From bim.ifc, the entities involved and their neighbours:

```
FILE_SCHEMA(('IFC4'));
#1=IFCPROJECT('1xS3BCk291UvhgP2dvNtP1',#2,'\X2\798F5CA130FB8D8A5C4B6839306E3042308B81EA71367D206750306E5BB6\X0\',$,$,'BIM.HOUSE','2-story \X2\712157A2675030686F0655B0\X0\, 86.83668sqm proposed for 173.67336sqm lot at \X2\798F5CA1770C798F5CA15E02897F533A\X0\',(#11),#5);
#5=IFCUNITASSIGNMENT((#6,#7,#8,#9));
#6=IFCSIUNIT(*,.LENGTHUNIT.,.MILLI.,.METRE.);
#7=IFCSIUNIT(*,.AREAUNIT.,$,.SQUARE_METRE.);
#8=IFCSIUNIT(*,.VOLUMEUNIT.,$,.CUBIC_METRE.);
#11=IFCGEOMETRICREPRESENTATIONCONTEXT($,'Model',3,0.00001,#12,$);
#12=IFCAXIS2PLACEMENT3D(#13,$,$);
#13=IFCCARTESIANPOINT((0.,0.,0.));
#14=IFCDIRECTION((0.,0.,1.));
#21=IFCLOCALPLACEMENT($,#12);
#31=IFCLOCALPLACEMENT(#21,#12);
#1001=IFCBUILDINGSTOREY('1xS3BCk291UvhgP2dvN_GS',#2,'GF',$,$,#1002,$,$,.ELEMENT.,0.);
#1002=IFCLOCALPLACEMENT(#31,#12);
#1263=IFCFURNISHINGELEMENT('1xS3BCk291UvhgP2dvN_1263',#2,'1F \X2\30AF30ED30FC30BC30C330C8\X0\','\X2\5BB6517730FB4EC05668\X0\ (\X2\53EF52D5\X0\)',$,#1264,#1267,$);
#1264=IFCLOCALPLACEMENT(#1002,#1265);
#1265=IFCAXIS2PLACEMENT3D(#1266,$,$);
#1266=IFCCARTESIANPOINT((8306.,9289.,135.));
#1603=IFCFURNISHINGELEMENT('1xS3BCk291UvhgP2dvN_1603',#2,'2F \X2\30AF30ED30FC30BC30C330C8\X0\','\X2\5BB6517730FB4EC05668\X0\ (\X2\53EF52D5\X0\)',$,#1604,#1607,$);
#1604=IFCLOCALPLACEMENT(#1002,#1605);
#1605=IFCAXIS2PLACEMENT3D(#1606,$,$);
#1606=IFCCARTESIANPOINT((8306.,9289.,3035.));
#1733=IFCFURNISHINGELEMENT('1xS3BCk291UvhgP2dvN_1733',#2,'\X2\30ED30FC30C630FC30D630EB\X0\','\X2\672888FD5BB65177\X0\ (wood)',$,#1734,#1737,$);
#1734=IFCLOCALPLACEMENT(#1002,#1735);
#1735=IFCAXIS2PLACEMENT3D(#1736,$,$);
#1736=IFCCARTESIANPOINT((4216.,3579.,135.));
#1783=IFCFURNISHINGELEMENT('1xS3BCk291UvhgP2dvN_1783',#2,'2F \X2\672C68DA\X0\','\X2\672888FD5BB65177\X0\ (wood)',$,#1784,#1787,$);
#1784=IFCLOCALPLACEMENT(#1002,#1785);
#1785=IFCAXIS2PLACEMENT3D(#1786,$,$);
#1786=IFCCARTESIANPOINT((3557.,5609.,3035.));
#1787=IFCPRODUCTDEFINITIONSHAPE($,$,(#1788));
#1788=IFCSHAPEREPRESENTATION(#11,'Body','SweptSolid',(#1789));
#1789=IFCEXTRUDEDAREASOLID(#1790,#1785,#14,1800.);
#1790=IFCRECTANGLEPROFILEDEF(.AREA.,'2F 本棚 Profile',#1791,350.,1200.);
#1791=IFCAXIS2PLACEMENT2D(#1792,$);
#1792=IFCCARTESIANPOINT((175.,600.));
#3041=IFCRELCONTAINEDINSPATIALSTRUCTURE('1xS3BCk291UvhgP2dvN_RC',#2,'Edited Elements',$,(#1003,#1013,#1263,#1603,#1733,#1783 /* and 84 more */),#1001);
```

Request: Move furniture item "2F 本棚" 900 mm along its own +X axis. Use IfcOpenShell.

```python
import ifcopenshell
import ifcopenshell.api.geometry
import ifcopenshell.util.placement

model = ifcopenshell.open("bim.ifc")

item = model.by_id(1783)
matrix = ifcopenshell.util.placement.get_local_placement(item.ObjectPlacement)
matrix[:3, 3] += matrix[:3, 0] * 900.0
ifcopenshell.api.geometry.edit_object_placement(model, product=item, matrix=matrix, is_si=False)

print(ifcopenshell.util.placement.get_local_placement(item.ObjectPlacement).round(3) + 0.0)

model.write("bim-out.ifc")
```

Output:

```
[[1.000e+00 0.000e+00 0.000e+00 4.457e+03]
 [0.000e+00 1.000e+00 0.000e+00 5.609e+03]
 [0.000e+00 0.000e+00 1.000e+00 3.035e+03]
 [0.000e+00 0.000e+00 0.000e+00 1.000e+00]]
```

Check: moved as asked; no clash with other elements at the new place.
